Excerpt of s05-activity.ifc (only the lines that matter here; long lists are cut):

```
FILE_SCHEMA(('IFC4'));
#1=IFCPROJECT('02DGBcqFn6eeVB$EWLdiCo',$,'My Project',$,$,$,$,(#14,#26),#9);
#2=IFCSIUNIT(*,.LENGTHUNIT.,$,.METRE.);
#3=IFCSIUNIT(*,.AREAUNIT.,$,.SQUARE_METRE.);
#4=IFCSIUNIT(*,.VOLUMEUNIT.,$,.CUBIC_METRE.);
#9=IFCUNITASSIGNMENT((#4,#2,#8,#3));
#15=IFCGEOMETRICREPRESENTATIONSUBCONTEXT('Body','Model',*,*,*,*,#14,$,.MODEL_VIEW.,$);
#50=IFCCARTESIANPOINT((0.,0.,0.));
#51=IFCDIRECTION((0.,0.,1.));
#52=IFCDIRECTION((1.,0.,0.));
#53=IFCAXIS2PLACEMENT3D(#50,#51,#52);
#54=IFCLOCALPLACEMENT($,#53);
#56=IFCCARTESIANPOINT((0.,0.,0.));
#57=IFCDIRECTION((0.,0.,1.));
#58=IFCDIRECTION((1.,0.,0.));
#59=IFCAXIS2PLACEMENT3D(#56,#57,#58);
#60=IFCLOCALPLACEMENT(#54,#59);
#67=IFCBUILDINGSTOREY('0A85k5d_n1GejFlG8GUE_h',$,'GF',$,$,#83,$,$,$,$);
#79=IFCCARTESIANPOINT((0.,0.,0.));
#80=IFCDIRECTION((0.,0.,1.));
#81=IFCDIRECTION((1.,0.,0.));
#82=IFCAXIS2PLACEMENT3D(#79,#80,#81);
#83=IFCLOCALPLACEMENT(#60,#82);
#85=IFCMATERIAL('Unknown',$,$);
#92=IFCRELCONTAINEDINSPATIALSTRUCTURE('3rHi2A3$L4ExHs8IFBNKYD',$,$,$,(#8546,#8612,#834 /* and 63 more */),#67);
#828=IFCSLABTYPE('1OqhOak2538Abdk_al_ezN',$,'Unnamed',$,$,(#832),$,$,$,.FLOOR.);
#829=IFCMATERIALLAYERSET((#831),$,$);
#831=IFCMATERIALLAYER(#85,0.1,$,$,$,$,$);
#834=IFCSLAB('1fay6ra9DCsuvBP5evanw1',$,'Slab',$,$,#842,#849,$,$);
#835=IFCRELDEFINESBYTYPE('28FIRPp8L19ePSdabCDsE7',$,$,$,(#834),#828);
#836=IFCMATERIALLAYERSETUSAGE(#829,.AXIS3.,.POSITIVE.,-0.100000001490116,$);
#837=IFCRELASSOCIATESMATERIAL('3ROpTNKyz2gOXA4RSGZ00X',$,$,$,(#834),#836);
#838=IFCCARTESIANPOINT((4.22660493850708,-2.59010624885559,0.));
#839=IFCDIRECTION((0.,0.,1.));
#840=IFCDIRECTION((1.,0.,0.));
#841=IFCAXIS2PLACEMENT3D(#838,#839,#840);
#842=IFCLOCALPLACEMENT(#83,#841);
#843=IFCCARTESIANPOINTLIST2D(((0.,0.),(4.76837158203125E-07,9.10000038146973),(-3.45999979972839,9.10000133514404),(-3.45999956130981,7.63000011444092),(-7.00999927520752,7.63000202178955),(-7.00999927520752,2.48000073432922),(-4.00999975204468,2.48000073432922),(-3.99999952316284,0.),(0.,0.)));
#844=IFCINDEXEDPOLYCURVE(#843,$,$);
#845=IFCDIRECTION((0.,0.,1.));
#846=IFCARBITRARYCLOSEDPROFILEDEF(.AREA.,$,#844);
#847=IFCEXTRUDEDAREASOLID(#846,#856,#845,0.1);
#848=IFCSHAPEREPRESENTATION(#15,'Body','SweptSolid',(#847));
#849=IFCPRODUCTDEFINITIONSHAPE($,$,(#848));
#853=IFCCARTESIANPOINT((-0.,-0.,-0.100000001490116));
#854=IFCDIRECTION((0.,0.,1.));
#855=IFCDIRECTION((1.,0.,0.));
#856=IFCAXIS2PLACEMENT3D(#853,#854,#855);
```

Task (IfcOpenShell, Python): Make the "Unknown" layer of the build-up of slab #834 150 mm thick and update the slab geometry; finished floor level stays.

```python
import ifcopenshell
import ifcopenshell.util.element
import ifcopenshell.util.representation

model = ifcopenshell.open("s05-activity.ifc")

layer_set = model.by_id(829)
layer = next(l for l in layer_set.MaterialLayers if l.Material and l.Material.Name == "Unknown")
change = 0.15 - layer.LayerThickness
layer.LayerThickness += change

# Geometry does not follow the layer set by itself.
slabs = [e for e in ifcopenshell.util.element.get_elements_by_material(model, layer_set) if e.is_a("IfcSlab")]
for slab in sorted(slabs, key=lambda e: e.id()):
    body = ifcopenshell.util.representation.get_representation(slab, "Model", "Body")
    solid = body.Items[0]
    old_depth = solid.Depth
    solid.Depth += change
    # Extruded upwards: lower the start of the extrusion so the top stays.
    x, y, z = solid.Position.Location.Coordinates
    solid.Position.Location = model.createIfcCartesianPoint((x, y, z - change))
    print(slab.id(), f"{old_depth:g} -> {solid.Depth:g}")

# The layers are counted up from the underside, which has moved.
for usage in {ifcopenshell.util.element.get_material(slab) for slab in slabs}:
    usage.OffsetFromReferenceLine -= change

model.write("s05-activity_updated.ifc")
```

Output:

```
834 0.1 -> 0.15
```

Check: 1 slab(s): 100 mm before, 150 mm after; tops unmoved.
